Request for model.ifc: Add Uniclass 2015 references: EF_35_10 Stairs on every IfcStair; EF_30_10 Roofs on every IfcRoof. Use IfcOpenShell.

First a look at what the model holds.

```python
import ifcopenshell

model = ifcopenshell.open("model.ifc")
print(model.schema)
print("classifications:", [c.Name for c in model.by_type("IfcClassification")])
for ifc_class in ("IfcDoor", "IfcRoof", "IfcStair", "IfcWall", "IfcWindow"):
    print(ifc_class, len(model.by_type(ifc_class)))
```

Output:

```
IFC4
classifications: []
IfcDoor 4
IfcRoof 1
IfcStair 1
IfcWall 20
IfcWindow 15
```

```python
import ifcopenshell
import ifcopenshell.api.classification

model = ifcopenshell.open("model.ifc")

system = ifcopenshell.api.classification.add_classification(model, classification="Uniclass 2015")

codes = {
    "IfcStair": ("EF_35_10", "Stairs"),
    "IfcRoof": ("EF_30_10", "Roofs"),
}
for ifc_class, (code, name) in codes.items():
    products = model.by_type(ifc_class)
    ifcopenshell.api.classification.add_reference(
        model, products=products, classification=system, identification=code, name=name
    )
    print(code, len(products))

model.write("model_v2.ifc")
```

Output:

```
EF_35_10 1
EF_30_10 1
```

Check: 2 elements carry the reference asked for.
